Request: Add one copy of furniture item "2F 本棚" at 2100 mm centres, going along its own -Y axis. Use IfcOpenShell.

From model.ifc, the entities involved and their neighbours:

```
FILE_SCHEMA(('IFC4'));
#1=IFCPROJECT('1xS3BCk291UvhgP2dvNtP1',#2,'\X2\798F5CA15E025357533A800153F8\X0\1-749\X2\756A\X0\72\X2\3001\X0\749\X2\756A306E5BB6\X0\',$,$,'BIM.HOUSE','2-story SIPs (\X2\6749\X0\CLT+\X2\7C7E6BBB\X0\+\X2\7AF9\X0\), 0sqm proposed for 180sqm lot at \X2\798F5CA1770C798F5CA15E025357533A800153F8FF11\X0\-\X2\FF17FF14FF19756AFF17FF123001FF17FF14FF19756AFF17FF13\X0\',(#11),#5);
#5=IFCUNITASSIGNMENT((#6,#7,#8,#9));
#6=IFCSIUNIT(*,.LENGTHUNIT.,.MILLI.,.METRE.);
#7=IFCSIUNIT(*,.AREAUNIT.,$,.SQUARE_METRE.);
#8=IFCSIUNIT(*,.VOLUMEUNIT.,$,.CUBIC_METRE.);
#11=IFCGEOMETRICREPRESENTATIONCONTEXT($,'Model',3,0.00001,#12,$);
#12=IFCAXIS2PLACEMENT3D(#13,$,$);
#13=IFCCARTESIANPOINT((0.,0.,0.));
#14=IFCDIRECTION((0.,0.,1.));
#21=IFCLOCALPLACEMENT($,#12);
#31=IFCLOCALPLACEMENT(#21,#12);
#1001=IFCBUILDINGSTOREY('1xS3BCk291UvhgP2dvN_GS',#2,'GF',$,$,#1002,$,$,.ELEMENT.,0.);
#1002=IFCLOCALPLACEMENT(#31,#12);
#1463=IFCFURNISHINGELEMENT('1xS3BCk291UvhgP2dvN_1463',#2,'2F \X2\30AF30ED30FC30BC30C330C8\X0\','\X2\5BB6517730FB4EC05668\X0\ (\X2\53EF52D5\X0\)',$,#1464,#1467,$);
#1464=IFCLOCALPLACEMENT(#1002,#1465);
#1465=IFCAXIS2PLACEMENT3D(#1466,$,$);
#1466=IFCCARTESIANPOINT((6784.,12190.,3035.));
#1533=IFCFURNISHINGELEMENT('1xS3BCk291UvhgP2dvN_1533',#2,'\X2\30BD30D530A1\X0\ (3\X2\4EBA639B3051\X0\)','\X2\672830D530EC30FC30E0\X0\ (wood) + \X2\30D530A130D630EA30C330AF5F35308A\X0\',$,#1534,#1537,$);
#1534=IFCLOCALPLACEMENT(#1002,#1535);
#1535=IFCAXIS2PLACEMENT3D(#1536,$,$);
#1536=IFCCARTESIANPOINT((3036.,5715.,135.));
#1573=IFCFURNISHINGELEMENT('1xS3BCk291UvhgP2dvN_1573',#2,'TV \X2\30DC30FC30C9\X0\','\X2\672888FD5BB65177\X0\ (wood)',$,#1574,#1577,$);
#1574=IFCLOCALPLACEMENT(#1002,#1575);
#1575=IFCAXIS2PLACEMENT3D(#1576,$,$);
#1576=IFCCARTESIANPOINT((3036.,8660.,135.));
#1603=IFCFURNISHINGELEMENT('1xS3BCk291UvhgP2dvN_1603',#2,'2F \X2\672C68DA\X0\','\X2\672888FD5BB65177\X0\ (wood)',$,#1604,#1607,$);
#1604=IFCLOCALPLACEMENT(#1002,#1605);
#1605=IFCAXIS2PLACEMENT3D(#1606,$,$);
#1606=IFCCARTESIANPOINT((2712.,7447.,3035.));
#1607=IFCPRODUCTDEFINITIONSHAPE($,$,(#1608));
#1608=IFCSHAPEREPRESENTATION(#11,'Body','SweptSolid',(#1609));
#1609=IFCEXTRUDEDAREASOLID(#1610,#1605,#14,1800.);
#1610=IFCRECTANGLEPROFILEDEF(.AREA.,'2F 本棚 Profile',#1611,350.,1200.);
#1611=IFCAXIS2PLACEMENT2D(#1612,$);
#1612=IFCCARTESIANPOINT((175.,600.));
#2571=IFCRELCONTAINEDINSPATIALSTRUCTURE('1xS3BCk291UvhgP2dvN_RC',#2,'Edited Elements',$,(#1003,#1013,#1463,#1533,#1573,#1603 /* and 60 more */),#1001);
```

```python
import ifcopenshell
import ifcopenshell.api.geometry
import ifcopenshell.api.root
import ifcopenshell.util.element
import ifcopenshell.util.placement
import ifcopenshell.util.unit

model = ifcopenshell.open("model.ifc")
unit_scale = ifcopenshell.util.unit.calculate_unit_scale(model)


def reuse_history(source, copy):
    """copy_class also copies each property set's owner history, people and application; keep the originals."""
    for rel in copy.IsDefinedBy:
        if rel.is_a("IfcRelDefinesByProperties") and (history := rel.RelatingPropertyDefinition.OwnerHistory):
            rel.RelatingPropertyDefinition.OwnerHistory = source.OwnerHistory
            ifcopenshell.util.element.remove_deep2(model, history)


source = model.by_id(1603)
base = ifcopenshell.util.placement.get_local_placement(source.ObjectPlacement)
step = -base[:3, 1] * 2.1 / unit_scale

for i in range(1, 2):
    copy = ifcopenshell.api.root.copy_class(model, product=source)
    copy.Representation = ifcopenshell.util.element.copy_deep(
        model, source.Representation, exclude=["IfcGeometricRepresentationContext", "IfcRepresentationMap"]
    )
    reuse_history(source, copy)
    matrix = base.copy()
    matrix[:3, 3] += i * step
    print("added at", matrix[:3, 3].round(3) + 0.0)
    ifcopenshell.api.geometry.edit_object_placement(model, product=copy, matrix=matrix, is_si=False)

model.write("model-out.ifc")
```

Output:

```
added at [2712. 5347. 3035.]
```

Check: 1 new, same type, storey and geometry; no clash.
